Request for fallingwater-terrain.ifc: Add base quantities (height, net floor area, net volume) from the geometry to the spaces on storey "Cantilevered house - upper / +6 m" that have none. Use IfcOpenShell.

First a look at what the model holds.

```python
import ifcopenshell
import ifcopenshell.util.element
import ifcopenshell.util.unit

model = ifcopenshell.open("fallingwater-terrain.ifc")
print(model.schema)
for unit_type in ("LENGTHUNIT", "AREAUNIT", "VOLUMEUNIT"):
    print(unit_type, ifcopenshell.util.unit.calculate_unit_scale(model, unit_type))
storey = next(s for s in model.by_type("IfcBuildingStorey") if s.Name == "Cantilevered house - upper / +6 m")
spaces = [e for e in ifcopenshell.util.element.get_decomposition(storey) if e.is_a("IfcSpace")]
for e in sorted(spaces, key=lambda e: e.id()):
    print(e.id(), e.is_a(), e.Name, list(ifcopenshell.util.element.get_psets(e, qtos_only=True)), sep=" | ")
```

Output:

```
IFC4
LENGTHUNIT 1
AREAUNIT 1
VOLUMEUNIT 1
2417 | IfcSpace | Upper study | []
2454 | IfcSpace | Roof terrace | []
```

```python
import ifcopenshell
import ifcopenshell.api.pset
import ifcopenshell.geom
import ifcopenshell.util.element
import ifcopenshell.util.shape
import ifcopenshell.util.unit

model = ifcopenshell.open("fallingwater-terrain.ifc")
unit_scale = ifcopenshell.util.unit.calculate_unit_scale(model)
area_scale = ifcopenshell.util.unit.calculate_unit_scale(model, "AREAUNIT")
volume_scale = ifcopenshell.util.unit.calculate_unit_scale(model, "VOLUMEUNIT")
settings = ifcopenshell.geom.settings()

storey = next(s for s in model.by_type("IfcBuildingStorey") if s.Name == "Cantilevered house - upper / +6 m")
spaces = [e for e in ifcopenshell.util.element.get_decomposition(storey) if e.is_a("IfcSpace")]

for e in sorted(spaces, key=lambda e: e.id()):
    if ifcopenshell.util.element.get_psets(e, qtos_only=True, should_inherit=False):
        continue
    # Geometry comes back in metres, in the element's own axes.
    shape = ifcopenshell.geom.create_shape(settings, e)
    values = {
        "Height": ifcopenshell.util.shape.get_z(shape.geometry) / unit_scale,
        "NetFloorArea": ifcopenshell.util.shape.get_footprint_area(shape.geometry) / area_scale,
        "NetVolume": ifcopenshell.util.shape.get_volume(shape.geometry) / volume_scale,
    }
    qto = ifcopenshell.api.pset.add_qto(model, product=e, name="Qto_SpaceBaseQuantities")
    ifcopenshell.api.pset.edit_qto(model, qto=qto, properties=values)
    print(e.id(), {k: round(v, 3) for k, v in values.items()})

model.write("fallingwater-terrain_rev.ifc")
```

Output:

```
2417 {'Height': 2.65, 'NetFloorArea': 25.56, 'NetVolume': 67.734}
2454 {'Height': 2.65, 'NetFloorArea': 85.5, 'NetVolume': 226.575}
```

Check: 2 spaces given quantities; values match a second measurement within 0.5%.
